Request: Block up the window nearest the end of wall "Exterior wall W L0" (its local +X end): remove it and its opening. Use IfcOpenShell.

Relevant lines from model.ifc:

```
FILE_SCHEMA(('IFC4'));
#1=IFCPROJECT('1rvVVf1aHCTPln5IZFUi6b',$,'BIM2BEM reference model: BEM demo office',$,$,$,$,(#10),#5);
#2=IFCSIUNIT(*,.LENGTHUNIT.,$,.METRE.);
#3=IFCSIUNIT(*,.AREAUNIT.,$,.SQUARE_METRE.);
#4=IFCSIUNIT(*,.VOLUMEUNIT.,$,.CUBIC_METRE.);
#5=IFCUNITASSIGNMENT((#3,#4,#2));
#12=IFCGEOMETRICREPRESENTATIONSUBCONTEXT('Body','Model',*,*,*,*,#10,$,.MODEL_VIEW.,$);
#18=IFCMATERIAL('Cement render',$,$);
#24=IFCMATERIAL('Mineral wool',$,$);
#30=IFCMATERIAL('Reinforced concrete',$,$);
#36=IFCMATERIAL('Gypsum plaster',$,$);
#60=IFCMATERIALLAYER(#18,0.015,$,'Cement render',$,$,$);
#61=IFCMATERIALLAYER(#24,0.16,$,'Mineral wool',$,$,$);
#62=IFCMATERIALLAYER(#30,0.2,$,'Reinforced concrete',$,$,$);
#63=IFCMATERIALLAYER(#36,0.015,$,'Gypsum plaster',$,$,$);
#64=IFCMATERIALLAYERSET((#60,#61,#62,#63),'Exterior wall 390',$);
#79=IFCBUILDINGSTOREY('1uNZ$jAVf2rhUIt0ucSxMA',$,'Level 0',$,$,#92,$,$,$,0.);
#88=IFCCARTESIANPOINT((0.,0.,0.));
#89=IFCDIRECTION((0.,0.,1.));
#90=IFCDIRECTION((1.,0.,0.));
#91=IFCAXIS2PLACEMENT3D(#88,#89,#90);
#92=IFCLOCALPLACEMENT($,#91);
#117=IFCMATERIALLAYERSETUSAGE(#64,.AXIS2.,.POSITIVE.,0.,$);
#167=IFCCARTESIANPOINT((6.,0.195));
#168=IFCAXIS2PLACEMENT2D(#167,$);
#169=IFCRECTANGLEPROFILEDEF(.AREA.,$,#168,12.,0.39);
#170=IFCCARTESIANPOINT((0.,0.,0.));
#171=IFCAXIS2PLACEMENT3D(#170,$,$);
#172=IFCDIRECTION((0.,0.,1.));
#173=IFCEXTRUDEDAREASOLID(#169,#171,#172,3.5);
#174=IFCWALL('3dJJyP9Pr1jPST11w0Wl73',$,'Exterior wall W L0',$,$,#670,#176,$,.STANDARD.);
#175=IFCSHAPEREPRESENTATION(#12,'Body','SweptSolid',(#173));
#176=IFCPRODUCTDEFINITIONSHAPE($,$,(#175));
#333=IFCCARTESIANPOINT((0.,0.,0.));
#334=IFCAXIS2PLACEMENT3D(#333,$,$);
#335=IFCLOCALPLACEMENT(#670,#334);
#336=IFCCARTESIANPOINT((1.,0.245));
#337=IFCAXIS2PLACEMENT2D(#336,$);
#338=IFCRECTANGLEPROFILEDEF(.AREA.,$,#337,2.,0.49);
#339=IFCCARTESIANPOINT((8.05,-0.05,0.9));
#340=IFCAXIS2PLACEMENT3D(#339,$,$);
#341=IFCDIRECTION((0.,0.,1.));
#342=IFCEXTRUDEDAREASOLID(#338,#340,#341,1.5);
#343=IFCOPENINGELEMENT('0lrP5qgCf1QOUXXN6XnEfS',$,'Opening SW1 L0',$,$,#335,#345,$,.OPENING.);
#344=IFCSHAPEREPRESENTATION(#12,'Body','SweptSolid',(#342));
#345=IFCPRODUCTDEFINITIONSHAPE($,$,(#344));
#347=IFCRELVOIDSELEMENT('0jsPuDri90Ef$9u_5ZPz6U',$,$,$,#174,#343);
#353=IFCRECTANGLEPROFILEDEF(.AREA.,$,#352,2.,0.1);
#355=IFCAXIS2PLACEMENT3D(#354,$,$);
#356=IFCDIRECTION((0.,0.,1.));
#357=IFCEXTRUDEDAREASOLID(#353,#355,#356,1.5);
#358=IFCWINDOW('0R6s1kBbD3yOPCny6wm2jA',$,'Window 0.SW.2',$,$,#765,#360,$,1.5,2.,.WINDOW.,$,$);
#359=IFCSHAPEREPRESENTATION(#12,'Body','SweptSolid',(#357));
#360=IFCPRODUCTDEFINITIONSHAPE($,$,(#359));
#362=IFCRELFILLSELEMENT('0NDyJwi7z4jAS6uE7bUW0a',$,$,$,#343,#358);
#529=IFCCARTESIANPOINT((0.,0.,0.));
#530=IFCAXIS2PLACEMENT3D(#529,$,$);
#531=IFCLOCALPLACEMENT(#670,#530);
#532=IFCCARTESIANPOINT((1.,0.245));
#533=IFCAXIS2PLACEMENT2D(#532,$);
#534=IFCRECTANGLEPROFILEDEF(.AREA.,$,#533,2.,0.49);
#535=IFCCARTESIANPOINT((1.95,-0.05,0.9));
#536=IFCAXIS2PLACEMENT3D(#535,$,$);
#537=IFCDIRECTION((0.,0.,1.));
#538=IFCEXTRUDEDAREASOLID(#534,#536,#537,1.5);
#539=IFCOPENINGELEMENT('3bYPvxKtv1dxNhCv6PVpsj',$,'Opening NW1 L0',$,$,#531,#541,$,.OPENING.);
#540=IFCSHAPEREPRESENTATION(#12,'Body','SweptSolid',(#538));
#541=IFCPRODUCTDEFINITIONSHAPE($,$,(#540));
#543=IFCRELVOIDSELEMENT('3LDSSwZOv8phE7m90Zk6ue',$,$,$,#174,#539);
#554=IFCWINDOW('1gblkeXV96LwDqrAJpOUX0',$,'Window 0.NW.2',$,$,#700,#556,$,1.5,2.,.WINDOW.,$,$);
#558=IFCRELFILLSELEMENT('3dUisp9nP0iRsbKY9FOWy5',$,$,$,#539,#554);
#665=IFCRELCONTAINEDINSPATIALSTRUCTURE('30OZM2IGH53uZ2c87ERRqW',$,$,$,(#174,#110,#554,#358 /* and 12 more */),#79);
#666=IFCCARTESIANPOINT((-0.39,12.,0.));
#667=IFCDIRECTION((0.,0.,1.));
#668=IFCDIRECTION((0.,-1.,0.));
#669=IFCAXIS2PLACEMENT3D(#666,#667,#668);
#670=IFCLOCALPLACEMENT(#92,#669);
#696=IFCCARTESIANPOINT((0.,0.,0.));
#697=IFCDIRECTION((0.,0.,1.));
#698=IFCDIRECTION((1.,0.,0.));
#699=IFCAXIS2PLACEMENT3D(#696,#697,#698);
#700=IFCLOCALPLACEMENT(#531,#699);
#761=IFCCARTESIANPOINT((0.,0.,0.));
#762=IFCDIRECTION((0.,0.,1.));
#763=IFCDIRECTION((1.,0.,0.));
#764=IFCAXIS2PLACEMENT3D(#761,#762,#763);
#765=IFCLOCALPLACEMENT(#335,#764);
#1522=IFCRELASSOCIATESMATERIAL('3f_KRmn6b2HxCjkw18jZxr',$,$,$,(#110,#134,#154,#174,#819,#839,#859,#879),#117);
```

```python
import ifcopenshell
import ifcopenshell.api.feature
import ifcopenshell.api.root
import ifcopenshell.geom
import ifcopenshell.util.shape

model = ifcopenshell.open("model.ifc")
settings = ifcopenshell.geom.settings()


def volume(element):
    """Net volume in cubic metres, openings subtracted."""
    shape = ifcopenshell.geom.create_shape(settings, element)
    return ifcopenshell.util.shape.get_volume(shape.geometry)


window = model.by_guid("0R6s1kBbD3yOPCny6wm2jA")
opening = window.FillsVoids[0].RelatingOpeningElement
wall = opening.VoidsElements[0].RelatingBuildingElement
before = volume(wall)

ifcopenshell.api.root.remove_product(model, product=window)
ifcopenshell.api.feature.remove_feature(model, feature=opening)

after = volume(wall)

print(f"wall volume {before:.3f} -> {after:.3f} m3")

model.write("model_v2.ifc")
```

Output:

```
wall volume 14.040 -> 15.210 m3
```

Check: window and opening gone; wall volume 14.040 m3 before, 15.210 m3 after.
